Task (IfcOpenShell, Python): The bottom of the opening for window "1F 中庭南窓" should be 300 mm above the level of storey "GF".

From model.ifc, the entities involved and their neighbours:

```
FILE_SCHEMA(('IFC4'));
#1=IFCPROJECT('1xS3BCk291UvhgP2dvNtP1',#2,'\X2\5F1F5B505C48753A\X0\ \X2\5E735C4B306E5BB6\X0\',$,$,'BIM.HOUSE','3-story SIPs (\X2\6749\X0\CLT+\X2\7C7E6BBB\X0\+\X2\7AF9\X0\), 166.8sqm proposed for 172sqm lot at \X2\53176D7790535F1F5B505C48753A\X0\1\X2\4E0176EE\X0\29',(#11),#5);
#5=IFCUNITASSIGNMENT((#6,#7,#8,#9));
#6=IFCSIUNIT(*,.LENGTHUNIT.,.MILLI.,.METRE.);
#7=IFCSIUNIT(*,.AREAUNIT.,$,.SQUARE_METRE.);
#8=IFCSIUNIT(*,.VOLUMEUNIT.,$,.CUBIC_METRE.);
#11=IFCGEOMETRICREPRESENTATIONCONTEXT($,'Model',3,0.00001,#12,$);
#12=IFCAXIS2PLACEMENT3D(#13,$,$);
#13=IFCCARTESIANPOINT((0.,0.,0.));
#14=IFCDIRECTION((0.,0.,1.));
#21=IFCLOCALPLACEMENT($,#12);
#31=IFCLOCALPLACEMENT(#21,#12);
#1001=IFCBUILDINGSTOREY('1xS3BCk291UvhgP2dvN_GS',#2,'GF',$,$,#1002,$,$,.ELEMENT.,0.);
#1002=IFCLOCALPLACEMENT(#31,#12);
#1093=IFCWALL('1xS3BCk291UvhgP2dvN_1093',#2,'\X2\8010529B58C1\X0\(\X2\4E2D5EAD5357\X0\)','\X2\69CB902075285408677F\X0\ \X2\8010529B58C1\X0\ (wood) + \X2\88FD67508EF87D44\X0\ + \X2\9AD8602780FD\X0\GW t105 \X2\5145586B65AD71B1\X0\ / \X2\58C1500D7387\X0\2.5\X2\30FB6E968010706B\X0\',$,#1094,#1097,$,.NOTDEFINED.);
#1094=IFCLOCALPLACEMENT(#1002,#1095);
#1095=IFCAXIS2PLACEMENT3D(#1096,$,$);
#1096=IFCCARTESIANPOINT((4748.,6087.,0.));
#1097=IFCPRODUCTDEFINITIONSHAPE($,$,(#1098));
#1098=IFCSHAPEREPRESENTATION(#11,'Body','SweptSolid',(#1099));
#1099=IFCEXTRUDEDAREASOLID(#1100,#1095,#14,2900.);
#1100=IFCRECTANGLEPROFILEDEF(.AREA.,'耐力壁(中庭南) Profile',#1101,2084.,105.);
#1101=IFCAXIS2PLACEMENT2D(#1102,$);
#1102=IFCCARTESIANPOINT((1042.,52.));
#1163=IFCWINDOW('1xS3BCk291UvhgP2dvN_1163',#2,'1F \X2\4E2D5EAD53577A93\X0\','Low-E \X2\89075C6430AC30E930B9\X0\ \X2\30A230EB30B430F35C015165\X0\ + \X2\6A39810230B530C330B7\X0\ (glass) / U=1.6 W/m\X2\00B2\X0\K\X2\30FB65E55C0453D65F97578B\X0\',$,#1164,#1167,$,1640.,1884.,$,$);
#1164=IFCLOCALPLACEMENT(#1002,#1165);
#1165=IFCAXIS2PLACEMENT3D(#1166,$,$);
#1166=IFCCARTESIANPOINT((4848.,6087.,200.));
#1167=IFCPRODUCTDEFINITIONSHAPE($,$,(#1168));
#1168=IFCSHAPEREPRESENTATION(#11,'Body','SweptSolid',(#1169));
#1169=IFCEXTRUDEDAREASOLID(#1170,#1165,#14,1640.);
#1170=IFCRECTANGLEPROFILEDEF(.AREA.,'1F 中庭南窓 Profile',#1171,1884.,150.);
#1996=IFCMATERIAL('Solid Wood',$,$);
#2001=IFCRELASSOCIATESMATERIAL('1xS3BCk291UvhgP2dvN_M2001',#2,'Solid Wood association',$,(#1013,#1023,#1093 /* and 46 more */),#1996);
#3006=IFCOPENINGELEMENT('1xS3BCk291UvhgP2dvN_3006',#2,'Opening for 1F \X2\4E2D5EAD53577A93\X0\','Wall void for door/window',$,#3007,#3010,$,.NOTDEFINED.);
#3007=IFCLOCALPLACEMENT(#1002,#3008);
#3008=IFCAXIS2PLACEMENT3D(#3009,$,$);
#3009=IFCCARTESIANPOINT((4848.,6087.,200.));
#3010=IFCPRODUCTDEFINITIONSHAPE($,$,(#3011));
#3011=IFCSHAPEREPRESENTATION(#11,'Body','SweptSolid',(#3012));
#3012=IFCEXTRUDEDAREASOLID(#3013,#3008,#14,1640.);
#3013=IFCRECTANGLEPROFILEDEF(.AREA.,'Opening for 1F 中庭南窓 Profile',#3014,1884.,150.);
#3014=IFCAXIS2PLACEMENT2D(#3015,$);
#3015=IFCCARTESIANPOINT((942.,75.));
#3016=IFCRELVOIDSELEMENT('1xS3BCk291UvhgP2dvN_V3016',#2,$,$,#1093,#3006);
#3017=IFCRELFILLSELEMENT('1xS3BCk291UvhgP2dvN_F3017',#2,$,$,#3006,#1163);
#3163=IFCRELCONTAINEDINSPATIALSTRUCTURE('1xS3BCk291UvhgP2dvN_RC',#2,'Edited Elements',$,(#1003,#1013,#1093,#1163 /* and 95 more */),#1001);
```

```python
import numpy as np
import ifcopenshell
import ifcopenshell.api.geometry
import ifcopenshell.geom
import ifcopenshell.util.element
import ifcopenshell.util.placement
import ifcopenshell.util.shape
import ifcopenshell.util.unit

model = ifcopenshell.open("model.ifc")
unit_scale = ifcopenshell.util.unit.calculate_unit_scale(model)

window = model.by_guid("1xS3BCk291UvhgP2dvN_1163")
opening = window.FillsVoids[0].RelatingOpeningElement
storey = ifcopenshell.util.element.get_container(window, ifc_class="IfcBuildingStorey")
level = ifcopenshell.util.placement.get_local_placement(storey.ObjectPlacement)[2, 3]

# The opening's origin need not be at the sill, so measure its lowest point.
shape = ifcopenshell.geom.create_shape(ifcopenshell.geom.settings(), opening)
bottom = ifcopenshell.util.shape.get_shape_bottom_elevation(shape, shape.geometry) / unit_scale
dz = level + 300.0 - bottom

shift = np.array([0.0, 0.0, dz])
# The window is not placed relative to its opening, so move both.
for product in (opening, window):
    matrix = ifcopenshell.util.placement.get_local_placement(product.ObjectPlacement)
    matrix[:3, 3] += shift
    ifcopenshell.api.geometry.edit_object_placement(model, product=product, matrix=matrix, is_si=False)

print(f"moved by {dz * unit_scale:+.3f} m")

model.write("model_rev.ifc")
```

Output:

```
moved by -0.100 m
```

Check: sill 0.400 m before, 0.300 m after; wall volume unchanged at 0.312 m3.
